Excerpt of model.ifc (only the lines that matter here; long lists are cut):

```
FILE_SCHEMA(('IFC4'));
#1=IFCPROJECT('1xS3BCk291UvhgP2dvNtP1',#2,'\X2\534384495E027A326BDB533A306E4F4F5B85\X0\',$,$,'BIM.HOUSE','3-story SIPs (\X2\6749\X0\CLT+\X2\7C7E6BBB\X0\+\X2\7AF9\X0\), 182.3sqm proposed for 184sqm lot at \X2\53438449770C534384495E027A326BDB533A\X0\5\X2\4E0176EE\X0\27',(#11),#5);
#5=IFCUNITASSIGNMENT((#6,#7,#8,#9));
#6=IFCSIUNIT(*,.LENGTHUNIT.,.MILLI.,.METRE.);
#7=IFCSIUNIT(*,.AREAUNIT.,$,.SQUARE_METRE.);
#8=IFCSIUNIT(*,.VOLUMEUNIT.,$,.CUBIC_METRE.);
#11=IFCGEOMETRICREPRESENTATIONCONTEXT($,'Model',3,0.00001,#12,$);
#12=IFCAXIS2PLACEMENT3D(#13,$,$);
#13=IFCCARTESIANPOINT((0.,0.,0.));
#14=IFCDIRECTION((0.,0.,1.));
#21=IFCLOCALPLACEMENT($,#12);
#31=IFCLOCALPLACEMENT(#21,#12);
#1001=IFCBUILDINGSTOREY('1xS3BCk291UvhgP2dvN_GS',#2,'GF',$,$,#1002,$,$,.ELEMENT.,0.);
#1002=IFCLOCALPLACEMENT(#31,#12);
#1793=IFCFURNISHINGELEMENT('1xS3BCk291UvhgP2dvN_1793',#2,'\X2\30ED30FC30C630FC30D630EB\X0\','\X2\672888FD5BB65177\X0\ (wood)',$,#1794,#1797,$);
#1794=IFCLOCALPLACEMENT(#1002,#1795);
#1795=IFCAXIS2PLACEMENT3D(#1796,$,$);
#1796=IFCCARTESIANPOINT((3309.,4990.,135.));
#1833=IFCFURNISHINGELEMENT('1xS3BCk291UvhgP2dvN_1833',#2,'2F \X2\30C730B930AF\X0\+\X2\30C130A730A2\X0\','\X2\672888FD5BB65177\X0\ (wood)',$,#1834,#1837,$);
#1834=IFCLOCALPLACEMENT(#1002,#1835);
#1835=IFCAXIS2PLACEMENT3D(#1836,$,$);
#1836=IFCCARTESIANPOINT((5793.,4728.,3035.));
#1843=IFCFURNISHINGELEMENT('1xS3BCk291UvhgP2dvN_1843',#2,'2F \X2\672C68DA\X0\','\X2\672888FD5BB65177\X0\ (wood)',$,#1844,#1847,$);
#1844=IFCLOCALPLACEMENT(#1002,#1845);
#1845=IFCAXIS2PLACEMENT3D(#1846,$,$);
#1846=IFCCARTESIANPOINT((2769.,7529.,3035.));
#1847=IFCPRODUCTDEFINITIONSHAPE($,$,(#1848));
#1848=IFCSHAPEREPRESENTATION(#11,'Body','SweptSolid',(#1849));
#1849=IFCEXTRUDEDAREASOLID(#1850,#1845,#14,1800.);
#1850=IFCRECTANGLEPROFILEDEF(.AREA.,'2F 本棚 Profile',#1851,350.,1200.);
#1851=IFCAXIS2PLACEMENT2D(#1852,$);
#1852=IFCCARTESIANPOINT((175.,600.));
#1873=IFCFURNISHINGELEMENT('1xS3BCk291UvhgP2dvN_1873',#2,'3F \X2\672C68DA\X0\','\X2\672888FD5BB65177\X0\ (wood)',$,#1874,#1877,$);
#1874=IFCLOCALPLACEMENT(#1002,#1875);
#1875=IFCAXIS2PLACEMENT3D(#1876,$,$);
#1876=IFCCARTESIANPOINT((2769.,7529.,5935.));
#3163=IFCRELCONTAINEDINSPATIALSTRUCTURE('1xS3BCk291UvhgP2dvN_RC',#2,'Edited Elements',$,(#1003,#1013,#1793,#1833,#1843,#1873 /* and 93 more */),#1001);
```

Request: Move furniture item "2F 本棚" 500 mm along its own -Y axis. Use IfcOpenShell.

```python
import ifcopenshell
import ifcopenshell.api.geometry
import ifcopenshell.util.placement
import ifcopenshell.util.unit

model = ifcopenshell.open("model.ifc")
unit_scale = ifcopenshell.util.unit.calculate_unit_scale(model)

item = model.by_guid("1xS3BCk291UvhgP2dvN_1843")
matrix = ifcopenshell.util.placement.get_local_placement(item.ObjectPlacement)
matrix[:3, 3] -= matrix[:3, 1] * 0.5 / unit_scale
ifcopenshell.api.geometry.edit_object_placement(model, product=item, matrix=matrix, is_si=False)

print(ifcopenshell.util.placement.get_local_placement(item.ObjectPlacement).round(3) + 0.0)

model.write("model_edited.ifc")
```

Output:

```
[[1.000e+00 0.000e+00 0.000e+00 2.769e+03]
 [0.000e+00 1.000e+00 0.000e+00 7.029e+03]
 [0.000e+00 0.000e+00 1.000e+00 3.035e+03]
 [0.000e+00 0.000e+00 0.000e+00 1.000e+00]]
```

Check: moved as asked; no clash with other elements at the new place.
